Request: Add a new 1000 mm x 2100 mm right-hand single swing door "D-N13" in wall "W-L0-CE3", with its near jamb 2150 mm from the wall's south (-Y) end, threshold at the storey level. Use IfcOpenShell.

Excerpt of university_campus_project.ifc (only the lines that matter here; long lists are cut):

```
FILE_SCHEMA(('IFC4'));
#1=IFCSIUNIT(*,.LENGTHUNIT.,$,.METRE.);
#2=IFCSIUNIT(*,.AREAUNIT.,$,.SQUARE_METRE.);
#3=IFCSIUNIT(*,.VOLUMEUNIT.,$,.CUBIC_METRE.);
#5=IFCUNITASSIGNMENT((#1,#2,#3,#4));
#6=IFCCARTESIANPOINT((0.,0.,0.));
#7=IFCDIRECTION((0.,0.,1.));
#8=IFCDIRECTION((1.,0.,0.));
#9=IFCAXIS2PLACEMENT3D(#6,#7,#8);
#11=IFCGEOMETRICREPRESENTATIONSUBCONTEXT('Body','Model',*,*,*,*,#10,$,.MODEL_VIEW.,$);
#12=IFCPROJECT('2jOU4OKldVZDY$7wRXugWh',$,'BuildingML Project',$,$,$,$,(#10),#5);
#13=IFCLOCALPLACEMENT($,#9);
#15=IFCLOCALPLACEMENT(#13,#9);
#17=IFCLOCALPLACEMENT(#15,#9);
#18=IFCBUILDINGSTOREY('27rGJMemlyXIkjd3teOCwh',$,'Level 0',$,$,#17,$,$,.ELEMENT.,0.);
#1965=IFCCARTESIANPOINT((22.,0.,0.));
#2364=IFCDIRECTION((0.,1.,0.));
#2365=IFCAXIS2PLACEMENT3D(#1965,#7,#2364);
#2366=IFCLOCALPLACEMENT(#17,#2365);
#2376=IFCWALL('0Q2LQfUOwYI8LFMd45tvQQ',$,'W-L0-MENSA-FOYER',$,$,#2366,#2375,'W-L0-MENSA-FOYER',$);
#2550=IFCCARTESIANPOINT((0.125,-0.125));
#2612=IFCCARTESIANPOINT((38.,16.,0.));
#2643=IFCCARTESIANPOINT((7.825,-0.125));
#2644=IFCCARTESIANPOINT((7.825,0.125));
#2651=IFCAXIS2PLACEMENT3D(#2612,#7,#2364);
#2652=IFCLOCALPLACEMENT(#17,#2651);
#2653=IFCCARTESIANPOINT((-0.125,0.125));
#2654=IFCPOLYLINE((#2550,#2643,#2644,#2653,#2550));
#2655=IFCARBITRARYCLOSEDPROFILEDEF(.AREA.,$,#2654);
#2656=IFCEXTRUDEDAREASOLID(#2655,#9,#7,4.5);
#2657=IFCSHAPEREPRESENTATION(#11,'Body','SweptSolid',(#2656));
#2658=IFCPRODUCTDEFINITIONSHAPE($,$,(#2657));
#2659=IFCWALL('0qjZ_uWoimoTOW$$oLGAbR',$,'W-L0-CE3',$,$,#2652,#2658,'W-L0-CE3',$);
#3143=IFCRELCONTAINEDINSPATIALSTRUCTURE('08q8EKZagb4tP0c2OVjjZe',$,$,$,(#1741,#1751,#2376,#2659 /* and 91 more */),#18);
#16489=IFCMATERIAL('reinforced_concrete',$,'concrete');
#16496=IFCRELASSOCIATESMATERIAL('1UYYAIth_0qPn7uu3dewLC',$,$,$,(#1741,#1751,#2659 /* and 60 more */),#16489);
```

```python
import numpy as np
import ifcopenshell
import ifcopenshell.api.feature
import ifcopenshell.api.geometry
import ifcopenshell.api.root
import ifcopenshell.api.spatial
import ifcopenshell.geom
import ifcopenshell.util.element
import ifcopenshell.util.placement
import ifcopenshell.util.representation
import ifcopenshell.util.shape
import ifcopenshell.util.unit

model = ifcopenshell.open("university_campus_project.ifc")
unit_scale = ifcopenshell.util.unit.calculate_unit_scale(model)
settings = ifcopenshell.geom.settings()


def volume(element):
    """Net volume in cubic metres, openings subtracted."""
    shape = ifcopenshell.geom.create_shape(settings, element)
    return ifcopenshell.util.shape.get_volume(shape.geometry)


wall = model.by_guid("0qjZ_uWoimoTOW$$oLGAbR")
storey = ifcopenshell.util.element.get_container(wall, ifc_class="IfcBuildingStorey")
context = ifcopenshell.util.representation.get_context(model, "Model", "Body", "MODEL_VIEW")
before = volume(wall)

width, height, from_end, sill = 1, 2.1, 2.15, 0.0  # metres

# The wall runs along its own X axis, and the end named is its -X end.
wall_shape = ifcopenshell.geom.create_shape(settings, wall)
x, y, z = ifcopenshell.util.shape.get_vertices(wall_shape.geometry).T
start = x.min() + from_end
face, thickness = float(y.min()), float(y.max() - y.min())
wall_matrix = ifcopenshell.util.placement.get_local_placement(wall.ObjectPlacement)
level = ifcopenshell.util.placement.get_local_placement(storey.ObjectPlacement)[2, 3]


def in_wall(x, y):
    """Placement at x, y metres in the wall's axes, at sill height."""
    matrix = wall_matrix.copy()
    matrix[:, 3] = wall_matrix @ np.array([x / unit_scale, y / unit_scale, 0.0, 1.0])
    matrix[2, 3] = level + sill / unit_scale
    return matrix


# Opening: a box that overshoots both wall faces by 50 mm.
opening = ifcopenshell.api.root.create_entity(model, ifc_class="IfcOpeningElement", predefined_type="OPENING")
box = ifcopenshell.api.geometry.add_wall_representation(
    model, context=context, length=width, height=height, thickness=thickness + 0.1
)
ifcopenshell.api.geometry.assign_representation(model, product=opening, representation=box)
ifcopenshell.api.geometry.edit_object_placement(model, product=opening, matrix=in_wall(start, face - 0.05), is_si=False)
ifcopenshell.api.feature.add_feature(model, feature=opening, element=wall)

door = ifcopenshell.api.root.create_entity(model, ifc_class="IfcDoor", name="D-N13", predefined_type="DOOR")
door.OverallWidth, door.OverallHeight = width / unit_scale, height / unit_scale
door.OperationType = "SINGLE_SWING_RIGHT"
body = ifcopenshell.api.geometry.add_door_representation(
    model,
    context=context,
    overall_width=door.OverallWidth,
    overall_height=door.OverallHeight,
    operation_type="SINGLE_SWING_RIGHT",
    lining_properties={"LiningDepth": thickness / unit_scale, "ThresholdDepth": thickness / unit_scale},
)
ifcopenshell.api.geometry.assign_representation(model, product=door, representation=body)
ifcopenshell.api.spatial.assign_container(model, products=[door], relating_structure=storey)
ifcopenshell.api.feature.add_filling(model, opening=opening, element=door)

# The lining spans the wall, so the door starts at the wall face.
ifcopenshell.api.geometry.edit_object_placement(model, product=door, matrix=in_wall(start, face), is_si=False)

after = volume(wall)

print(f"wall volume {before:.3f} -> {after:.3f} m3")

model.write("university_campus_project_v2.ifc")
```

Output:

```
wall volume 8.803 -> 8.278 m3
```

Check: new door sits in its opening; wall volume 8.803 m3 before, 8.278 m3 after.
